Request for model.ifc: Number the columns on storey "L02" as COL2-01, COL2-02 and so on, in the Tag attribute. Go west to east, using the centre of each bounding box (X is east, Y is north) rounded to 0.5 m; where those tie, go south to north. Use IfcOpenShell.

First a look at what the model holds.

```python
import ifcopenshell
import ifcopenshell.util.element
import ifcopenshell.util.placement

model = ifcopenshell.open("model.ifc")
print(model.schema)
storey = next(s for s in model.by_type("IfcBuildingStorey") if s.Name == "L02")
columns = [e for e in ifcopenshell.util.element.get_decomposition(storey) if e.is_a("IfcColumn")]
for e in sorted(columns, key=lambda e: e.id()):
    origin = ifcopenshell.util.placement.get_local_placement(e.ObjectPlacement)[:3, 3]
    print(e.id(), e.Tag, e.Name, origin.round(2) + 0.0, sep=" | ")
```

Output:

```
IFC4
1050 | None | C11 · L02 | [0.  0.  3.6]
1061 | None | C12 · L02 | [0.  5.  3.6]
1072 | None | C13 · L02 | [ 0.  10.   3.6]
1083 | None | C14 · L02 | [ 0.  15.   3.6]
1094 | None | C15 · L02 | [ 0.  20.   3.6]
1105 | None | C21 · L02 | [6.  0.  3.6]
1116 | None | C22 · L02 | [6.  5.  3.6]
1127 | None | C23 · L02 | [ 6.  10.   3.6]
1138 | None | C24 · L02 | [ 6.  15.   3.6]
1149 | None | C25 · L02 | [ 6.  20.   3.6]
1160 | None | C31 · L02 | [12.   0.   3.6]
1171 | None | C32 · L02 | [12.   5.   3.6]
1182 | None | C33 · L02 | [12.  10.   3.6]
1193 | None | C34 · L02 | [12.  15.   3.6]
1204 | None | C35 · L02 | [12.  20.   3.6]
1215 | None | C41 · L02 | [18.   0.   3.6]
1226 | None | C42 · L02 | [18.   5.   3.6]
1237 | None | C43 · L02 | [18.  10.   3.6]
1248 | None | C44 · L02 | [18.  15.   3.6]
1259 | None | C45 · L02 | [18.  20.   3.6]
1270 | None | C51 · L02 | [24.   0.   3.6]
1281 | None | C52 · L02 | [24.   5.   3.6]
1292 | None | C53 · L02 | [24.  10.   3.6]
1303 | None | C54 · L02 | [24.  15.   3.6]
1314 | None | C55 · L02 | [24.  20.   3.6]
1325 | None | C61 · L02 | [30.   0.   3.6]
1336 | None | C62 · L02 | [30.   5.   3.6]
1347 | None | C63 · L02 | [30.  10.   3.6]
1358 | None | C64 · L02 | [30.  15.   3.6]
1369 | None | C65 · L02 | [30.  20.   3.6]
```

```python
import ifcopenshell
import ifcopenshell.geom
import ifcopenshell.util.element
import ifcopenshell.util.shape

model = ifcopenshell.open("model.ifc")
settings = ifcopenshell.geom.settings()
settings.set("use-world-coords", True)


def centre(element):
    shape = ifcopenshell.geom.create_shape(settings, element)
    return ifcopenshell.util.shape.get_bbox_centroid(shape.geometry)


storey = next(s for s in model.by_type("IfcBuildingStorey") if s.Name == "L02")
columns = [e for e in ifcopenshell.util.element.get_decomposition(storey) if e.is_a("IfcColumn")]

# Insertion points can sit at a corner or the storey origin, so sort by the geometry (in metres).
centres = {e: centre(e) for e in columns}
columns.sort(key=lambda e: (round(centres[e][0] / 0.5), centres[e][1]))

for i, e in enumerate(columns, start=1):
    number = f"COL2-{i:02d}"
    e.Tag = number
    print(e.id(), number)

model.write("model_edited.ifc")
```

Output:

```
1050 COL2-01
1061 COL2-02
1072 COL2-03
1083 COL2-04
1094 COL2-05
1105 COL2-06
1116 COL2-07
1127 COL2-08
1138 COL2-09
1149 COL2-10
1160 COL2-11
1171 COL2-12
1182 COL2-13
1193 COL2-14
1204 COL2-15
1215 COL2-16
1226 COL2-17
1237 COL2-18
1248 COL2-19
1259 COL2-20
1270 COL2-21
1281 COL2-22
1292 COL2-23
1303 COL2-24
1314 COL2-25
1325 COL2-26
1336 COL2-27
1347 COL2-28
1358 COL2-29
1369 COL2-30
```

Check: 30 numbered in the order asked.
